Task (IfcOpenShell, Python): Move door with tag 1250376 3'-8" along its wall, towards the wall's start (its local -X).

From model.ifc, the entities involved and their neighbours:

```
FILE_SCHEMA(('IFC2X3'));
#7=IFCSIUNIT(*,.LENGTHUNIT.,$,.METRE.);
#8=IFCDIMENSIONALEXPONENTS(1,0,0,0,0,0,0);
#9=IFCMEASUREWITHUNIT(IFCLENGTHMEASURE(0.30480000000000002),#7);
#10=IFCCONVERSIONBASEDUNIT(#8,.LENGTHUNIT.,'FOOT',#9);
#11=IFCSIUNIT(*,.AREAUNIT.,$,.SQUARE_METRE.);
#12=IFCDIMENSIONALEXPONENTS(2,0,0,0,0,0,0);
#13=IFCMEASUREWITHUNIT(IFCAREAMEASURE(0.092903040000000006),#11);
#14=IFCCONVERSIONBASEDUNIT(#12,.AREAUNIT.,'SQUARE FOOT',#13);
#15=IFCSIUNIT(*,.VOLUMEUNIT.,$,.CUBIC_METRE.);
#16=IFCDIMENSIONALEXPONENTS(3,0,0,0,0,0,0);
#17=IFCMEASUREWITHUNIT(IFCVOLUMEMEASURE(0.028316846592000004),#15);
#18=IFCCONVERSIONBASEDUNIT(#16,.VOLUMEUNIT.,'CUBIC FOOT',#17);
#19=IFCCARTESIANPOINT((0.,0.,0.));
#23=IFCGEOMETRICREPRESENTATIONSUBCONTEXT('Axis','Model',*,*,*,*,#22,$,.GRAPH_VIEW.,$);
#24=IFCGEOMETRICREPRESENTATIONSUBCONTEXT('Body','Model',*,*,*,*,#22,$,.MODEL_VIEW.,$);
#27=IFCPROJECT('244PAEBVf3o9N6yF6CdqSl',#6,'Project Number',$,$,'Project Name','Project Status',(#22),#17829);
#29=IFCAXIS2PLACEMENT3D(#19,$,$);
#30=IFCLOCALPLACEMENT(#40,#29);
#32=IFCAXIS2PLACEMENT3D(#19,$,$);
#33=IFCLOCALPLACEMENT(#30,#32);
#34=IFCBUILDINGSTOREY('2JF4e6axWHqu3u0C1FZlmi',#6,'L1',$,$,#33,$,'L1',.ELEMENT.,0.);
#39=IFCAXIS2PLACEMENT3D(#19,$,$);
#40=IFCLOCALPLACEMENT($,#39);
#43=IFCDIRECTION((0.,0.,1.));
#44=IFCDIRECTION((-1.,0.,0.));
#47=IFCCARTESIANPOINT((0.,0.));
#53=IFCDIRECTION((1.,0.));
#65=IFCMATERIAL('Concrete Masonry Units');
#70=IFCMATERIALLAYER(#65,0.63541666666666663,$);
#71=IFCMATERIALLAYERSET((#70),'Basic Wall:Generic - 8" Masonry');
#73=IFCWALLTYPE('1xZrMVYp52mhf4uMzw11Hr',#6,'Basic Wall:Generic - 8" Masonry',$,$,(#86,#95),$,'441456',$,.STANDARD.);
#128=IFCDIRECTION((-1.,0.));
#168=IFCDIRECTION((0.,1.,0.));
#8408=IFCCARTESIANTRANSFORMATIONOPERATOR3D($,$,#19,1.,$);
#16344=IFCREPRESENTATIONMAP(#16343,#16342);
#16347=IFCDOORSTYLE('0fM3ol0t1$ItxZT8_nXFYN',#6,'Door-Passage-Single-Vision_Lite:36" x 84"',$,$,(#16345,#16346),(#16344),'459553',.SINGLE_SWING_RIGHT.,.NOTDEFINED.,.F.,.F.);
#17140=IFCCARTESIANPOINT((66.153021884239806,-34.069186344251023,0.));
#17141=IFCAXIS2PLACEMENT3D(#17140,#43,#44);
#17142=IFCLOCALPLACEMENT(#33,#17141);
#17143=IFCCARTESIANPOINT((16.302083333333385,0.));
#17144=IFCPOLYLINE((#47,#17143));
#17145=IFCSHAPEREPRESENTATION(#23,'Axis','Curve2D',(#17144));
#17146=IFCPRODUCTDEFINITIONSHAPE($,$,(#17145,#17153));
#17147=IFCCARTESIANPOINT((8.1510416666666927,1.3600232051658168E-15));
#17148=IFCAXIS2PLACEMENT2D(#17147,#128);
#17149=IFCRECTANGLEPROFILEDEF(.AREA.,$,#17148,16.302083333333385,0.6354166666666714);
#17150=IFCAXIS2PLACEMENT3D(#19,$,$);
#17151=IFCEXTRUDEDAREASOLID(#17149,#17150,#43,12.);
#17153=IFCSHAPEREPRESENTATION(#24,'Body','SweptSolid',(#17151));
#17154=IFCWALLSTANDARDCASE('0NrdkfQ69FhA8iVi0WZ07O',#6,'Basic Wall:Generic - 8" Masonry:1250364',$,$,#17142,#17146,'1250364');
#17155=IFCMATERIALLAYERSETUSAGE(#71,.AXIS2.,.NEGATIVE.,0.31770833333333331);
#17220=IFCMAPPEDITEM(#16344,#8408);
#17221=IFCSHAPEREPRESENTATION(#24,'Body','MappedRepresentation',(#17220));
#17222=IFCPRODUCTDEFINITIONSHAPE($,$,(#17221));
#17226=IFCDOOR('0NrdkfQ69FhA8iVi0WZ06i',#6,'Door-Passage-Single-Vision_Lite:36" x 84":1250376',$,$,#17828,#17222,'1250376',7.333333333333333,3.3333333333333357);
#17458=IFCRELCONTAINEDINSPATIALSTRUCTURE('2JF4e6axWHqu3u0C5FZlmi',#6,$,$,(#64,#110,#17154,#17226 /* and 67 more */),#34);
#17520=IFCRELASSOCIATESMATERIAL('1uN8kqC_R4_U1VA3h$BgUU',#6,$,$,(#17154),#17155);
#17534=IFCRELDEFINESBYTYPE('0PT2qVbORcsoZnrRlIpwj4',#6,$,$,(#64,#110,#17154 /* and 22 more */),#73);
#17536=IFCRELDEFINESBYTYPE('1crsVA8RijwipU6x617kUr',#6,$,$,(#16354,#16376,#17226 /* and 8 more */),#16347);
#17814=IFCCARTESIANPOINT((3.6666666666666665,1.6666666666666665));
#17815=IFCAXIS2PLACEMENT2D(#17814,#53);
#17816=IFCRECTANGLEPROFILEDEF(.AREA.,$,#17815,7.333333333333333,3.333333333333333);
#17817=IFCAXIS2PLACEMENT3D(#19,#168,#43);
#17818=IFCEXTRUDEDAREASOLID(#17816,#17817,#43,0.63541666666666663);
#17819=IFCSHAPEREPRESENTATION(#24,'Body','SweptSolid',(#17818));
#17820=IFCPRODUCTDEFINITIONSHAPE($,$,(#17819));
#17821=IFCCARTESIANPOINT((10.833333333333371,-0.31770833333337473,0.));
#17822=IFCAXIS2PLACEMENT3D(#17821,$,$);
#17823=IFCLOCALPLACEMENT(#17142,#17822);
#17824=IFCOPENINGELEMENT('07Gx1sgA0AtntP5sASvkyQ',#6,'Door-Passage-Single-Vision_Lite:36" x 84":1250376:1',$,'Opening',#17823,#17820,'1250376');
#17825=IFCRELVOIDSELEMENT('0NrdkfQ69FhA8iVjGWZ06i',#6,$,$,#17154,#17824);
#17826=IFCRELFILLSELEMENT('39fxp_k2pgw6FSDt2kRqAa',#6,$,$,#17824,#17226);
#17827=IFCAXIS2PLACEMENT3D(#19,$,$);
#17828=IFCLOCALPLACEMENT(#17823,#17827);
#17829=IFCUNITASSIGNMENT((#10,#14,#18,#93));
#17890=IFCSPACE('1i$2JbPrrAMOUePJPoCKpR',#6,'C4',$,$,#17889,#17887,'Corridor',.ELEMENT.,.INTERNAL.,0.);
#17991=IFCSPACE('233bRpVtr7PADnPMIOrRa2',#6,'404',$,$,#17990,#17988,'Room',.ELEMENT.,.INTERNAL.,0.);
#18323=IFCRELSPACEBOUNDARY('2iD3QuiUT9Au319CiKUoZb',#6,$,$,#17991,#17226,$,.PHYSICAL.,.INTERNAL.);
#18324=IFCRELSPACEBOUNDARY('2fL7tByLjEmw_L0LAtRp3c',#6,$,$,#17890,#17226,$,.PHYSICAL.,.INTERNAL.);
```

```python
import ifcopenshell
import ifcopenshell.api.geometry
import ifcopenshell.util.placement
import ifcopenshell.util.unit

model = ifcopenshell.open("model.ifc")
unit_scale = ifcopenshell.util.unit.calculate_unit_scale(model)

door = model.by_guid("0NrdkfQ69FhA8iVi0WZ06i")
opening = door.FillsVoids[0].RelatingOpeningElement
wall = opening.VoidsElements[0].RelatingBuildingElement

wall_matrix = ifcopenshell.util.placement.get_local_placement(wall.ObjectPlacement)
shift = wall_matrix[:3, 0] * -44 * 0.0254 / unit_scale
before = ifcopenshell.util.placement.get_local_placement(door.ObjectPlacement)[:3, 3].copy()

# The door is placed relative to its opening, so it follows when the opening moves.
matrix = ifcopenshell.util.placement.get_local_placement(opening.ObjectPlacement)
matrix[:3, 3] += shift
ifcopenshell.api.geometry.edit_object_placement(
    model, product=opening, matrix=matrix, is_si=False, should_transform_children=True
)

after = ifcopenshell.util.placement.get_local_placement(door.ObjectPlacement)[:3, 3]
print("door moved by", (after - before).round(3) + 0.0)

model.write("model_updated.ifc")
```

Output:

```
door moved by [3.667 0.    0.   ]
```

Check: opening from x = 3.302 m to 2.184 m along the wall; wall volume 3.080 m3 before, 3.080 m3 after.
